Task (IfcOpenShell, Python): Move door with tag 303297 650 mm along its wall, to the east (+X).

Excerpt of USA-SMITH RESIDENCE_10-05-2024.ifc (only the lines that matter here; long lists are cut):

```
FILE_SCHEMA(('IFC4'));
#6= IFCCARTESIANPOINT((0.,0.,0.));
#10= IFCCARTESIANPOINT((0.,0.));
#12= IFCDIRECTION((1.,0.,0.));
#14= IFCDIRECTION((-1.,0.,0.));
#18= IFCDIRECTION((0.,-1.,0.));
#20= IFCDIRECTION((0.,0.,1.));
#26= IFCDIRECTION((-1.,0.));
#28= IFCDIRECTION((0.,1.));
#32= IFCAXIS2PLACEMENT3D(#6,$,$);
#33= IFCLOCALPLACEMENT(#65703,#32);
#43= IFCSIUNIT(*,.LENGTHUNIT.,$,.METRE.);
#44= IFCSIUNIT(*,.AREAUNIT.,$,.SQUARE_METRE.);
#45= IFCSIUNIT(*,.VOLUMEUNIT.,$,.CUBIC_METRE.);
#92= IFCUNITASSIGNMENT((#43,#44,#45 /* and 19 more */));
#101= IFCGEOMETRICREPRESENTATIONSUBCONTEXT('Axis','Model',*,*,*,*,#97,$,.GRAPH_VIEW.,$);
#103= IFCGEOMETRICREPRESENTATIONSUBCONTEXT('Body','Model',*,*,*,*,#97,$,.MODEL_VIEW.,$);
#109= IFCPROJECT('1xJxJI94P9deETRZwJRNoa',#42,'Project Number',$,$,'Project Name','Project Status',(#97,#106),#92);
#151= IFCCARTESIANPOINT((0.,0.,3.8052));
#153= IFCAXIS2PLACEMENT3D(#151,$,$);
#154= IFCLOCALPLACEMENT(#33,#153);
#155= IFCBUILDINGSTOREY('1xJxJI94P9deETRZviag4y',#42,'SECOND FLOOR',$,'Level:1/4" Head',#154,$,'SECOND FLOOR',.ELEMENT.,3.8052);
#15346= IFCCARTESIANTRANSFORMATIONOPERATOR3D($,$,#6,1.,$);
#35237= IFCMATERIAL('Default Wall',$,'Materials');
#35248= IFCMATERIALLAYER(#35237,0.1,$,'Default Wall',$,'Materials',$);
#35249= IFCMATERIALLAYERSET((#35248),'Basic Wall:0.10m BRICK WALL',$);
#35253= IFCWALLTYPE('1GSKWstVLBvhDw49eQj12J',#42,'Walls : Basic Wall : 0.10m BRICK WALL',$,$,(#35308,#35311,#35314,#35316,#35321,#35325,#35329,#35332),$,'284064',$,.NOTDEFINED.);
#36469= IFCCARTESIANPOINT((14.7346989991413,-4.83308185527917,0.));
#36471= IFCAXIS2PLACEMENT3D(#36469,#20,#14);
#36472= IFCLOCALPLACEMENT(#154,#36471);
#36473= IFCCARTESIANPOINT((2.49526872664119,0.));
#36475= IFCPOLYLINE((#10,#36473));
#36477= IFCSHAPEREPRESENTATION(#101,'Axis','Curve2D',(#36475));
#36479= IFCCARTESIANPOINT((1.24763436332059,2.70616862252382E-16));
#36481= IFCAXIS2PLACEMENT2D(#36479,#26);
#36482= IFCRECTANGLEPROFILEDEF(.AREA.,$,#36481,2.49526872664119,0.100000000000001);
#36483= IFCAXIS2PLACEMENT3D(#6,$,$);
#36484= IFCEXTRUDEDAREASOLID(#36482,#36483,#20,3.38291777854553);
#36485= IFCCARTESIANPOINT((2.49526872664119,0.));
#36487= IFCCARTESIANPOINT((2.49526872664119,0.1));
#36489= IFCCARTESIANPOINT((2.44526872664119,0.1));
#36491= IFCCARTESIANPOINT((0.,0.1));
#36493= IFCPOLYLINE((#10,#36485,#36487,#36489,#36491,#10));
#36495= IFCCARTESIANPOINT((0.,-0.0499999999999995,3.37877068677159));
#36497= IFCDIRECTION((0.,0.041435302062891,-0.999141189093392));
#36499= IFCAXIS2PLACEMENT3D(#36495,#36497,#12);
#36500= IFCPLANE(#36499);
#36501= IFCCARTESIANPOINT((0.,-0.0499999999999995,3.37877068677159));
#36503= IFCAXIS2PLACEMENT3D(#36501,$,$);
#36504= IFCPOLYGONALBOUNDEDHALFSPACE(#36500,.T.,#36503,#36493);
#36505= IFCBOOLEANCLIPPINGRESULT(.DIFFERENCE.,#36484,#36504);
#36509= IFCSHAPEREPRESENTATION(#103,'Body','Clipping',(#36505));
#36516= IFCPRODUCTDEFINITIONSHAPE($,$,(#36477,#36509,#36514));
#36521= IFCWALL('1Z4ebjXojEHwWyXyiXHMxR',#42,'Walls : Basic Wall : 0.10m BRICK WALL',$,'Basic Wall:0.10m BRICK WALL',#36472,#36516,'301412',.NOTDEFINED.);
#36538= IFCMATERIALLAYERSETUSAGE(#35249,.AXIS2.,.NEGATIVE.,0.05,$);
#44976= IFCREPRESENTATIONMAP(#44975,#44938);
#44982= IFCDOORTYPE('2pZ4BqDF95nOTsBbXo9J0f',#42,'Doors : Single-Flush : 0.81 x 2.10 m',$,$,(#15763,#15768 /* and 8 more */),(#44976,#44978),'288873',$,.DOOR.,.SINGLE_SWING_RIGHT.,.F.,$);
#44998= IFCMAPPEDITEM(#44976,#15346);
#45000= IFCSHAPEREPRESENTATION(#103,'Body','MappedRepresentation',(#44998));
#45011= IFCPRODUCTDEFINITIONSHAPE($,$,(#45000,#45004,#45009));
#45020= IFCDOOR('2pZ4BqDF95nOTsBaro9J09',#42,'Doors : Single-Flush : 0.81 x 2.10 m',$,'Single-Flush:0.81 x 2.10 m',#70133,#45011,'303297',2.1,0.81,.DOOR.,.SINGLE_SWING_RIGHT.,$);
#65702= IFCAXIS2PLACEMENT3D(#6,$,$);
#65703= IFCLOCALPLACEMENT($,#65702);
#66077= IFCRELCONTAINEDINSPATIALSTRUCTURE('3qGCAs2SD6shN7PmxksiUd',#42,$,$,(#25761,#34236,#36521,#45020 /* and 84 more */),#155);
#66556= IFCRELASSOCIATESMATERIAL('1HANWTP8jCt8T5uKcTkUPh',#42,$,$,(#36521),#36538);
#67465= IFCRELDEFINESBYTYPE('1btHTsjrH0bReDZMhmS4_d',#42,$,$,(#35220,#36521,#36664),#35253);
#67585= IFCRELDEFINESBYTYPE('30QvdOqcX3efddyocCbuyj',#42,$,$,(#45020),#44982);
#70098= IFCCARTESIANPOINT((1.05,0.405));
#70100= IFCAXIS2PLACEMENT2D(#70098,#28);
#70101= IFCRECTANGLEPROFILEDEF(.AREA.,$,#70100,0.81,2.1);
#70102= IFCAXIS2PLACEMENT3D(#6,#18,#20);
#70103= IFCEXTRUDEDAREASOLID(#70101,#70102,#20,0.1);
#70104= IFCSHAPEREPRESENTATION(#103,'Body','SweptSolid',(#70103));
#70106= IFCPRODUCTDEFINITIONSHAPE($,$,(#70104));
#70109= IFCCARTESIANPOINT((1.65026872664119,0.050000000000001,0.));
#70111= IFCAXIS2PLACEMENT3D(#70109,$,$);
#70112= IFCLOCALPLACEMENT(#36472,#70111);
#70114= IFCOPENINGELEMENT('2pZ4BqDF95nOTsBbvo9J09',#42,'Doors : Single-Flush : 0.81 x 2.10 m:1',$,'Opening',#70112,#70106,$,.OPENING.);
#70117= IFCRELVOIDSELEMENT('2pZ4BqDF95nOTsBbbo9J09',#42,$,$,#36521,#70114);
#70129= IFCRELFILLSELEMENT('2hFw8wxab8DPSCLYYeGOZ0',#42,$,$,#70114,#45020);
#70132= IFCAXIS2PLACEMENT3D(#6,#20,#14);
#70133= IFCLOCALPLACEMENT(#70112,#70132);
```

```python
import ifcopenshell
import ifcopenshell.api.geometry
import ifcopenshell.util.placement

model = ifcopenshell.open("USA-SMITH RESIDENCE_10-05-2024.ifc")

door = model.by_id(45020)
opening = door.FillsVoids[0].RelatingOpeningElement
wall = opening.VoidsElements[0].RelatingBuildingElement

wall_matrix = ifcopenshell.util.placement.get_local_placement(wall.ObjectPlacement)
shift = wall_matrix[:3, 0] * -0.65
before = ifcopenshell.util.placement.get_local_placement(door.ObjectPlacement)[:3, 3].copy()

# The door is placed relative to its opening, so it follows when the opening moves.
matrix = ifcopenshell.util.placement.get_local_placement(opening.ObjectPlacement)
matrix[:3, 3] += shift
ifcopenshell.api.geometry.edit_object_placement(
    model, product=opening, matrix=matrix, is_si=False, should_transform_children=True
)

after = ifcopenshell.util.placement.get_local_placement(door.ObjectPlacement)[:3, 3]
print("door moved by", (after - before).round(3) + 0.0)

model.write("USA-SMITH RESIDENCE_10-05-2024_rev.ifc")
```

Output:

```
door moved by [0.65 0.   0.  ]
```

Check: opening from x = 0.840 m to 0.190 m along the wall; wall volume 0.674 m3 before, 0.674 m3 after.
